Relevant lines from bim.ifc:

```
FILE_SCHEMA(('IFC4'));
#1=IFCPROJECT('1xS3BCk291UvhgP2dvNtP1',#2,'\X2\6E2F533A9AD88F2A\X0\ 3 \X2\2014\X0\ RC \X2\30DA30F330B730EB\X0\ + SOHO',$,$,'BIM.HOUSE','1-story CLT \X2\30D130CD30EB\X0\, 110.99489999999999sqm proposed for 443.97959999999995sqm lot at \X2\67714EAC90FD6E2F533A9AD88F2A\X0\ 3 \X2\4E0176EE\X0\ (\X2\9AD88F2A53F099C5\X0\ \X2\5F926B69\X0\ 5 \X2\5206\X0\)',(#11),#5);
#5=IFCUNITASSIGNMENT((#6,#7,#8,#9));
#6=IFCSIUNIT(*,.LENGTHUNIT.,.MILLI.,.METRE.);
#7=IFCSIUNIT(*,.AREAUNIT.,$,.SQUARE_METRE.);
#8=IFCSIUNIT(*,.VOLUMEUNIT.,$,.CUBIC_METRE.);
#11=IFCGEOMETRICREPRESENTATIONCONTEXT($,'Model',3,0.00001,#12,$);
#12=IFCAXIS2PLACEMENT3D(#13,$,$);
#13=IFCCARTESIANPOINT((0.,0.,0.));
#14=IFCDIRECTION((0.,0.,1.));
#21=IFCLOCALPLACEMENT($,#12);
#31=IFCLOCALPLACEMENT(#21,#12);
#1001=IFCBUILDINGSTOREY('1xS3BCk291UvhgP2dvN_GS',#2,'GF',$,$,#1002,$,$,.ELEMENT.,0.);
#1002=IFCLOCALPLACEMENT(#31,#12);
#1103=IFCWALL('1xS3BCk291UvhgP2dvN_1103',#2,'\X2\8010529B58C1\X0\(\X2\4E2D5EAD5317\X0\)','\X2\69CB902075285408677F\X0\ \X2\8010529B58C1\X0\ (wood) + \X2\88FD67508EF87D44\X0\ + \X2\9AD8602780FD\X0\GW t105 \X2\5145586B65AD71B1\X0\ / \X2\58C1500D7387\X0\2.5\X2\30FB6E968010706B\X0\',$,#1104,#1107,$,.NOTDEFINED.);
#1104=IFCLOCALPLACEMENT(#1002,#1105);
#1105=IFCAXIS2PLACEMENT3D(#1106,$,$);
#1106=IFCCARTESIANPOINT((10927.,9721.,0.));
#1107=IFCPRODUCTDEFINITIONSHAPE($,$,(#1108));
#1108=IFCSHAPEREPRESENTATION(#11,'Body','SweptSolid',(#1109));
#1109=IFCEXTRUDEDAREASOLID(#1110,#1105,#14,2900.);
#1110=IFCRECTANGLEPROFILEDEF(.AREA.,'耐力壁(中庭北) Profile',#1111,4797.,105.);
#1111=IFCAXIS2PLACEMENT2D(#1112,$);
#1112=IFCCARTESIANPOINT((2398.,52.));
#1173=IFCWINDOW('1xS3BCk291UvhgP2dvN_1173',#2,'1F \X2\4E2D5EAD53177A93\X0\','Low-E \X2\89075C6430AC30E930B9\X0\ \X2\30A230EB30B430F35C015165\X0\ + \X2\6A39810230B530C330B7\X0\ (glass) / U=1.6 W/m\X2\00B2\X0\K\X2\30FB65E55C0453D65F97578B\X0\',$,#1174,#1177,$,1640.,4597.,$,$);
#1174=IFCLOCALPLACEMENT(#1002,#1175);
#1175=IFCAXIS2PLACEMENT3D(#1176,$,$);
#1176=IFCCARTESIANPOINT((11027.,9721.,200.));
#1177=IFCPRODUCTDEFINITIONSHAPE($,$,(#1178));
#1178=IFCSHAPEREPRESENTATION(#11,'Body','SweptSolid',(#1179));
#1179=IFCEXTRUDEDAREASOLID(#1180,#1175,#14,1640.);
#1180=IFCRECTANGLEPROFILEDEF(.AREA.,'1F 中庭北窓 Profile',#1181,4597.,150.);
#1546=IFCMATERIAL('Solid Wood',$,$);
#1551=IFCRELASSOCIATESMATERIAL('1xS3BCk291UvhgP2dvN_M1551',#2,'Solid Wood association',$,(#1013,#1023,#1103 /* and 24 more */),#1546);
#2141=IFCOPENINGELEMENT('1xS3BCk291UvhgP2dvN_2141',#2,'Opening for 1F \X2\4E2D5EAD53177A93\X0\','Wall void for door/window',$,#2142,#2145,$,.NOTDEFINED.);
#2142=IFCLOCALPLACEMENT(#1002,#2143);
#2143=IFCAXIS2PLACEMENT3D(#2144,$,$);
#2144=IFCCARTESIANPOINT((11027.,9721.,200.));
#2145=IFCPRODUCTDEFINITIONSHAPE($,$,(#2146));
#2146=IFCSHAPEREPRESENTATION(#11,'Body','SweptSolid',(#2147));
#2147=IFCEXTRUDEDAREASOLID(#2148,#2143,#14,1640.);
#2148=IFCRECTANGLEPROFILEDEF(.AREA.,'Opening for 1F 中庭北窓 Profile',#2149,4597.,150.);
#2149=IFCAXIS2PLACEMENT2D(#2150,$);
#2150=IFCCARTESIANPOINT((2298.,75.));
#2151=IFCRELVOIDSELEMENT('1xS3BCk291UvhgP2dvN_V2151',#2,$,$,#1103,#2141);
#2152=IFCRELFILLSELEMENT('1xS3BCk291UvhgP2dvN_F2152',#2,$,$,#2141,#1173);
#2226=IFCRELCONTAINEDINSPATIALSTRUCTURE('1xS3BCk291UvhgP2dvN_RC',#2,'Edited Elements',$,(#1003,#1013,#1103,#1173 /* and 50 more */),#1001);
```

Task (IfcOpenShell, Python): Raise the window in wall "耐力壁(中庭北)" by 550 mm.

```python
import numpy as np
import ifcopenshell
import ifcopenshell.api.geometry
import ifcopenshell.util.placement
import ifcopenshell.util.unit

model = ifcopenshell.open("bim.ifc")
unit_scale = ifcopenshell.util.unit.calculate_unit_scale(model)

window = model.by_guid("1xS3BCk291UvhgP2dvN_1173")
opening = window.FillsVoids[0].RelatingOpeningElement
dz = 0.55 / unit_scale

shift = np.array([0.0, 0.0, dz])
# The window is not placed relative to its opening, so move both.
for product in (opening, window):
    matrix = ifcopenshell.util.placement.get_local_placement(product.ObjectPlacement)
    matrix[:3, 3] += shift
    ifcopenshell.api.geometry.edit_object_placement(model, product=product, matrix=matrix, is_si=False)

print(f"moved by {dz * unit_scale:+.3f} m")

model.write("bim_edited.ifc")
```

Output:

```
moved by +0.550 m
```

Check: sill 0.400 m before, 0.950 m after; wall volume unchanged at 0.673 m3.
